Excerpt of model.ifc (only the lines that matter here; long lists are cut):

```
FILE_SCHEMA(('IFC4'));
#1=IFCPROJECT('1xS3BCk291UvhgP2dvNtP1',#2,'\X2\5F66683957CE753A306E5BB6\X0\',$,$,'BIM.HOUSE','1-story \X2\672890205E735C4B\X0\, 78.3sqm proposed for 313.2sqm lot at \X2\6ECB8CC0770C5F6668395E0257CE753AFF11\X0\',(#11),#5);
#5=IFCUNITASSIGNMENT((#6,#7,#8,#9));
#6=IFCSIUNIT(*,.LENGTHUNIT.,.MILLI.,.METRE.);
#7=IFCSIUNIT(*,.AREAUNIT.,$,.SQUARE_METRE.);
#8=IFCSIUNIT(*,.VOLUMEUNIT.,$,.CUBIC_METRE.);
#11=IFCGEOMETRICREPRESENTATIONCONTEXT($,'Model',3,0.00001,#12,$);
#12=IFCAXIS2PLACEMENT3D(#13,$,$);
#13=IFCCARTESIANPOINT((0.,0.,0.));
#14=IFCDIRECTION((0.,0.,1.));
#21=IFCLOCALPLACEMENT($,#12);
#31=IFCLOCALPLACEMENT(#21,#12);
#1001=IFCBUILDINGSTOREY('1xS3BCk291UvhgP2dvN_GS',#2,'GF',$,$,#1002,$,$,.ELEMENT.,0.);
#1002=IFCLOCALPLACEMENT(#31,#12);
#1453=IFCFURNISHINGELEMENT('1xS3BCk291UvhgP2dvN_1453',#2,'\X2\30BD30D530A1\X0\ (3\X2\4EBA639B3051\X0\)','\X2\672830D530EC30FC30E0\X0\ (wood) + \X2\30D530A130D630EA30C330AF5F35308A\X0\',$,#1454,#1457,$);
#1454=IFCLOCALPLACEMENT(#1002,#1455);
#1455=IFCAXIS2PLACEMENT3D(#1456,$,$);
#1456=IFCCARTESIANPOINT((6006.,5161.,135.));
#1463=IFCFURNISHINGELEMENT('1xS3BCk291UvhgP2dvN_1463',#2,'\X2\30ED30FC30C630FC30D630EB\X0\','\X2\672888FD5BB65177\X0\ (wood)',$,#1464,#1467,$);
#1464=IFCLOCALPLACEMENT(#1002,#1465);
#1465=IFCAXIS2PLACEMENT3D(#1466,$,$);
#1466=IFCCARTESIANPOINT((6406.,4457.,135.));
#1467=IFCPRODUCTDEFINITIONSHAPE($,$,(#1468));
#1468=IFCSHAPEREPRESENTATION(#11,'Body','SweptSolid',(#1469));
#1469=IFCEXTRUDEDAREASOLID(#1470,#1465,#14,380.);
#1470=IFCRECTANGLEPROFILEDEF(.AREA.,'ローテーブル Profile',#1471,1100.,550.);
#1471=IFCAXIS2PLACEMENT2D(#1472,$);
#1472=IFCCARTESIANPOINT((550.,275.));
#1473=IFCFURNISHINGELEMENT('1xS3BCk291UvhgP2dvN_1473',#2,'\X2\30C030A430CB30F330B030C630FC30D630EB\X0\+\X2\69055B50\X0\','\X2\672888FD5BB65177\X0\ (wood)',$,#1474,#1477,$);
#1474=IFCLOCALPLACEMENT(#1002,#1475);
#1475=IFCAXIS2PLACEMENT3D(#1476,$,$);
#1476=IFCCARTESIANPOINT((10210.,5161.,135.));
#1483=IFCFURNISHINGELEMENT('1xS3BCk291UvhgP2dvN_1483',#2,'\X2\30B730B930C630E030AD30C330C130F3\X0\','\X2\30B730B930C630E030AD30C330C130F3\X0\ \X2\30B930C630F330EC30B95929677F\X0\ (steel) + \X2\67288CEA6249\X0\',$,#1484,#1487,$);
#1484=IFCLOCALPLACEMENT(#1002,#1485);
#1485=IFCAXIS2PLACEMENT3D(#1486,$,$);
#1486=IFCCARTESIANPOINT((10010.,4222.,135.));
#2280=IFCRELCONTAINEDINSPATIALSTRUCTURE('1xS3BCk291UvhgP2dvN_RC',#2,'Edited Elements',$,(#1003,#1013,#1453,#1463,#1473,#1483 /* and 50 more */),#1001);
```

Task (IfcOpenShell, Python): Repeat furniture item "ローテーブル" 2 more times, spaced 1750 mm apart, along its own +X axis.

```python
import ifcopenshell
import ifcopenshell.api.geometry
import ifcopenshell.api.root
import ifcopenshell.util.element
import ifcopenshell.util.placement
import ifcopenshell.util.unit

model = ifcopenshell.open("model.ifc")
unit_scale = ifcopenshell.util.unit.calculate_unit_scale(model)


def reuse_history(source, copy):
    """copy_class also copies each property set's owner history, people and application; keep the originals."""
    for rel in copy.IsDefinedBy:
        if rel.is_a("IfcRelDefinesByProperties") and (history := rel.RelatingPropertyDefinition.OwnerHistory):
            rel.RelatingPropertyDefinition.OwnerHistory = source.OwnerHistory
            ifcopenshell.util.element.remove_deep2(model, history)


source = model.by_guid("1xS3BCk291UvhgP2dvN_1463")
base = ifcopenshell.util.placement.get_local_placement(source.ObjectPlacement)
step = base[:3, 0] * 1.75 / unit_scale

for i in range(1, 3):
    copy = ifcopenshell.api.root.copy_class(model, product=source)
    copy.Representation = ifcopenshell.util.element.copy_deep(
        model, source.Representation, exclude=["IfcGeometricRepresentationContext", "IfcRepresentationMap"]
    )
    reuse_history(source, copy)
    matrix = base.copy()
    matrix[:3, 3] += i * step
    print("added at", matrix[:3, 3].round(3) + 0.0)
    ifcopenshell.api.geometry.edit_object_placement(model, product=copy, matrix=matrix, is_si=False)

model.write("model_edited.ifc")
```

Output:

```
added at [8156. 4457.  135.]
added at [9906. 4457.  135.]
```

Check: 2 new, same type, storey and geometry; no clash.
